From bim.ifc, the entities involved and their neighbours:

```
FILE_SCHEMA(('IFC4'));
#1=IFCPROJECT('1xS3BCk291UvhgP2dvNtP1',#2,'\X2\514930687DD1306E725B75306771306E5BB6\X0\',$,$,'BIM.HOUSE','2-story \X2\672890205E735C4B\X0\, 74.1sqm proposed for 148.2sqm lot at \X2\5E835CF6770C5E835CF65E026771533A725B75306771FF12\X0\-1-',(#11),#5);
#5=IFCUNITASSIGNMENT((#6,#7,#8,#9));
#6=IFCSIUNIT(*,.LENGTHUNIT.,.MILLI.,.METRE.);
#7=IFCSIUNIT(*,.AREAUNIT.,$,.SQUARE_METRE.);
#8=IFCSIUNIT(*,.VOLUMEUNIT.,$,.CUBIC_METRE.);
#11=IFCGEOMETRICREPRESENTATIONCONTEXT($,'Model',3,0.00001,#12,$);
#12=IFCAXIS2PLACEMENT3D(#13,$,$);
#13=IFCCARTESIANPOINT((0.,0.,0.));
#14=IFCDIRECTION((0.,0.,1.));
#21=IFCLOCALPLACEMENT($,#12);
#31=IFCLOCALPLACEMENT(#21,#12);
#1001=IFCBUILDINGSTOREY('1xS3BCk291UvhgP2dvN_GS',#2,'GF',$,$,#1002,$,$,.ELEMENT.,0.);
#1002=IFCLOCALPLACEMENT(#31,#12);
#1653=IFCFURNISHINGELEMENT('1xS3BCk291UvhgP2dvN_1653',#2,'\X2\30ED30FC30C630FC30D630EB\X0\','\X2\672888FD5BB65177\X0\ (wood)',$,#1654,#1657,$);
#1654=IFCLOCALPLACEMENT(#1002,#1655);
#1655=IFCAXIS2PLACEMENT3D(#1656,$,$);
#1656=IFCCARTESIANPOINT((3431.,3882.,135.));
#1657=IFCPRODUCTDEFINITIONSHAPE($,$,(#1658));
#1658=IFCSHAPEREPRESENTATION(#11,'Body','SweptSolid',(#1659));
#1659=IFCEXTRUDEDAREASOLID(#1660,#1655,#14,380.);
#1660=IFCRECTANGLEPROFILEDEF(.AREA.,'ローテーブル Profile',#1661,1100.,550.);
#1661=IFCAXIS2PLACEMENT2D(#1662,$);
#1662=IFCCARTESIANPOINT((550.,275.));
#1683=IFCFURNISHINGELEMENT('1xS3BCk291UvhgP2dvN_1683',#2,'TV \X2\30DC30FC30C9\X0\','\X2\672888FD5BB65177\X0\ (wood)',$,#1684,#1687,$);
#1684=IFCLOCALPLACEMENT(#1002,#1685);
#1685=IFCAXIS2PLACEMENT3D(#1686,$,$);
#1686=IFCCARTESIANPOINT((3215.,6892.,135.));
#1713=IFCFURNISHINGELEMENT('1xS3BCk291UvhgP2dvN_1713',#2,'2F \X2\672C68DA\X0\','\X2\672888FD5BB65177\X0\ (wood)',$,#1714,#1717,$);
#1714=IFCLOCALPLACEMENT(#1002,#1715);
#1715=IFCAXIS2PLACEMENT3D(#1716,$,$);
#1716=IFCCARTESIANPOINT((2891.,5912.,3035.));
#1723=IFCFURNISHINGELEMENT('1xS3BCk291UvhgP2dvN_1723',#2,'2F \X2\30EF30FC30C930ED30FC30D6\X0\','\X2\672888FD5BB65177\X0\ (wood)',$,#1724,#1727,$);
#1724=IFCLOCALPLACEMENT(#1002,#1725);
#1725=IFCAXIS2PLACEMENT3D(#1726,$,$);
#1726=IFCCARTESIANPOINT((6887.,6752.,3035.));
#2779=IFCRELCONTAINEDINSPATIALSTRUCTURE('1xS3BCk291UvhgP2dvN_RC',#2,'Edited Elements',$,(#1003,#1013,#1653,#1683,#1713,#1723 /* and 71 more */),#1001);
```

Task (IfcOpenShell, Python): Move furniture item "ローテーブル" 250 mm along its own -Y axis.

```python
import ifcopenshell
import ifcopenshell.api.geometry
import ifcopenshell.util.placement
import ifcopenshell.util.unit

model = ifcopenshell.open("bim.ifc")
unit_scale = ifcopenshell.util.unit.calculate_unit_scale(model)

item = model.by_guid("1xS3BCk291UvhgP2dvN_1653")
matrix = ifcopenshell.util.placement.get_local_placement(item.ObjectPlacement)
matrix[:3, 3] -= matrix[:3, 1] * 0.25 / unit_scale
ifcopenshell.api.geometry.edit_object_placement(model, product=item, matrix=matrix, is_si=False)

print(ifcopenshell.util.placement.get_local_placement(item.ObjectPlacement).round(3) + 0.0)

model.write("bim-out.ifc")
```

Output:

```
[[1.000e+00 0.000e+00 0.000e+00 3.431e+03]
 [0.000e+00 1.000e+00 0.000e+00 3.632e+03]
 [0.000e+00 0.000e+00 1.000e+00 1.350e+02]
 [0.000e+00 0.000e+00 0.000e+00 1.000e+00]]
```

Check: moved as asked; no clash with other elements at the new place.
